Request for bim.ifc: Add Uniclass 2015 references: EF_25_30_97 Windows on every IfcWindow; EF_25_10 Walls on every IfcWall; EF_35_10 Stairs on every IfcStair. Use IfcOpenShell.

First a look at what the model holds.

```python
import ifcopenshell

model = ifcopenshell.open("bim.ifc")
print(model.schema)
print("classifications:", [c.Name for c in model.by_type("IfcClassification")])
for ifc_class in ("IfcDoor", "IfcRoof", "IfcStair", "IfcWall", "IfcWindow"):
    print(ifc_class, len(model.by_type(ifc_class)))
```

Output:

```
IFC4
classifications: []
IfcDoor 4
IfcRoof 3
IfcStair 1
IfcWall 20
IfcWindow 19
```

```python
import ifcopenshell
import ifcopenshell.api.classification

model = ifcopenshell.open("bim.ifc")

system = ifcopenshell.api.classification.add_classification(model, classification="Uniclass 2015")

codes = {
    "IfcWindow": ("EF_25_30_97", "Windows"),
    "IfcWall": ("EF_25_10", "Walls"),
    "IfcStair": ("EF_35_10", "Stairs"),
}
for ifc_class, (code, name) in codes.items():
    products = model.by_type(ifc_class)
    ifcopenshell.api.classification.add_reference(
        model, products=products, classification=system, identification=code, name=name
    )
    print(code, len(products))

model.write("bim-out.ifc")
```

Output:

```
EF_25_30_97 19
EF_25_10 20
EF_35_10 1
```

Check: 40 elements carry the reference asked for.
